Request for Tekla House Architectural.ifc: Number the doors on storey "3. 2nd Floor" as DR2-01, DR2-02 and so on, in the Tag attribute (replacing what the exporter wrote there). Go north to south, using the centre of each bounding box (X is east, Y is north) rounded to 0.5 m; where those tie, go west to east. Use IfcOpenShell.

First a look at what the model holds.

```python
import ifcopenshell
import ifcopenshell.util.element
import ifcopenshell.util.placement

model = ifcopenshell.open("Tekla House Architectural.ifc")
print(model.schema)
storey = next(s for s in model.by_type("IfcBuildingStorey") if s.Name == "3. 2nd Floor")
doors = [e for e in ifcopenshell.util.element.get_decomposition(storey) if e.is_a("IfcDoor")]
for e in sorted(doors, key=lambda e: e.id()):
    origin = ifcopenshell.util.placement.get_local_placement(e.ObjectPlacement)[:3, 3]
    print(e.id(), e.Tag, e.Name, origin.round(2) + 0.0, sep=" | ")
```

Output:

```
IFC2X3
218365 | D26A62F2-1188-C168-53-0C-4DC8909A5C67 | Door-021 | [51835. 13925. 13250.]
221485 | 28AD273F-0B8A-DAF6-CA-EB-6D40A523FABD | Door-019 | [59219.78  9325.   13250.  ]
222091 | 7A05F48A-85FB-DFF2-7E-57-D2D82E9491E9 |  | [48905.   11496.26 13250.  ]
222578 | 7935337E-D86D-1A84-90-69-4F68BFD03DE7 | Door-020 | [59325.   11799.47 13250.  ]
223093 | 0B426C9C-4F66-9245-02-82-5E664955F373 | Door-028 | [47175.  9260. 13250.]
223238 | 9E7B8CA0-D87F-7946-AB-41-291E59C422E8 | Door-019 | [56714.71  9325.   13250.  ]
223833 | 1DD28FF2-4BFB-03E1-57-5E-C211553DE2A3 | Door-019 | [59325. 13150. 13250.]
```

```python
import ifcopenshell
import ifcopenshell.geom
import ifcopenshell.util.element
import ifcopenshell.util.shape

model = ifcopenshell.open("Tekla House Architectural.ifc")
settings = ifcopenshell.geom.settings()
settings.set("use-world-coords", True)


def centre(element):
    shape = ifcopenshell.geom.create_shape(settings, element)
    return ifcopenshell.util.shape.get_bbox_centroid(shape.geometry)


storey = next(s for s in model.by_type("IfcBuildingStorey") if s.Name == "3. 2nd Floor")
doors = [e for e in ifcopenshell.util.element.get_decomposition(storey) if e.is_a("IfcDoor")]

# Insertion points can sit at a corner or the storey origin, so sort by the geometry (in metres).
centres = {e: centre(e) for e in doors}
doors.sort(key=lambda e: (-round(centres[e][1] / 0.5), centres[e][0]))

for i, e in enumerate(doors, start=1):
    number = f"DR2-{i:02d}"
    e.Tag = number
    print(e.id(), number)

model.write("Tekla House Architectural_updated.ifc")
```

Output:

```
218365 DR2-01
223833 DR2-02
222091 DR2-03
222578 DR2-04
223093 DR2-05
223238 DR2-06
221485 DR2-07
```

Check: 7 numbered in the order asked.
